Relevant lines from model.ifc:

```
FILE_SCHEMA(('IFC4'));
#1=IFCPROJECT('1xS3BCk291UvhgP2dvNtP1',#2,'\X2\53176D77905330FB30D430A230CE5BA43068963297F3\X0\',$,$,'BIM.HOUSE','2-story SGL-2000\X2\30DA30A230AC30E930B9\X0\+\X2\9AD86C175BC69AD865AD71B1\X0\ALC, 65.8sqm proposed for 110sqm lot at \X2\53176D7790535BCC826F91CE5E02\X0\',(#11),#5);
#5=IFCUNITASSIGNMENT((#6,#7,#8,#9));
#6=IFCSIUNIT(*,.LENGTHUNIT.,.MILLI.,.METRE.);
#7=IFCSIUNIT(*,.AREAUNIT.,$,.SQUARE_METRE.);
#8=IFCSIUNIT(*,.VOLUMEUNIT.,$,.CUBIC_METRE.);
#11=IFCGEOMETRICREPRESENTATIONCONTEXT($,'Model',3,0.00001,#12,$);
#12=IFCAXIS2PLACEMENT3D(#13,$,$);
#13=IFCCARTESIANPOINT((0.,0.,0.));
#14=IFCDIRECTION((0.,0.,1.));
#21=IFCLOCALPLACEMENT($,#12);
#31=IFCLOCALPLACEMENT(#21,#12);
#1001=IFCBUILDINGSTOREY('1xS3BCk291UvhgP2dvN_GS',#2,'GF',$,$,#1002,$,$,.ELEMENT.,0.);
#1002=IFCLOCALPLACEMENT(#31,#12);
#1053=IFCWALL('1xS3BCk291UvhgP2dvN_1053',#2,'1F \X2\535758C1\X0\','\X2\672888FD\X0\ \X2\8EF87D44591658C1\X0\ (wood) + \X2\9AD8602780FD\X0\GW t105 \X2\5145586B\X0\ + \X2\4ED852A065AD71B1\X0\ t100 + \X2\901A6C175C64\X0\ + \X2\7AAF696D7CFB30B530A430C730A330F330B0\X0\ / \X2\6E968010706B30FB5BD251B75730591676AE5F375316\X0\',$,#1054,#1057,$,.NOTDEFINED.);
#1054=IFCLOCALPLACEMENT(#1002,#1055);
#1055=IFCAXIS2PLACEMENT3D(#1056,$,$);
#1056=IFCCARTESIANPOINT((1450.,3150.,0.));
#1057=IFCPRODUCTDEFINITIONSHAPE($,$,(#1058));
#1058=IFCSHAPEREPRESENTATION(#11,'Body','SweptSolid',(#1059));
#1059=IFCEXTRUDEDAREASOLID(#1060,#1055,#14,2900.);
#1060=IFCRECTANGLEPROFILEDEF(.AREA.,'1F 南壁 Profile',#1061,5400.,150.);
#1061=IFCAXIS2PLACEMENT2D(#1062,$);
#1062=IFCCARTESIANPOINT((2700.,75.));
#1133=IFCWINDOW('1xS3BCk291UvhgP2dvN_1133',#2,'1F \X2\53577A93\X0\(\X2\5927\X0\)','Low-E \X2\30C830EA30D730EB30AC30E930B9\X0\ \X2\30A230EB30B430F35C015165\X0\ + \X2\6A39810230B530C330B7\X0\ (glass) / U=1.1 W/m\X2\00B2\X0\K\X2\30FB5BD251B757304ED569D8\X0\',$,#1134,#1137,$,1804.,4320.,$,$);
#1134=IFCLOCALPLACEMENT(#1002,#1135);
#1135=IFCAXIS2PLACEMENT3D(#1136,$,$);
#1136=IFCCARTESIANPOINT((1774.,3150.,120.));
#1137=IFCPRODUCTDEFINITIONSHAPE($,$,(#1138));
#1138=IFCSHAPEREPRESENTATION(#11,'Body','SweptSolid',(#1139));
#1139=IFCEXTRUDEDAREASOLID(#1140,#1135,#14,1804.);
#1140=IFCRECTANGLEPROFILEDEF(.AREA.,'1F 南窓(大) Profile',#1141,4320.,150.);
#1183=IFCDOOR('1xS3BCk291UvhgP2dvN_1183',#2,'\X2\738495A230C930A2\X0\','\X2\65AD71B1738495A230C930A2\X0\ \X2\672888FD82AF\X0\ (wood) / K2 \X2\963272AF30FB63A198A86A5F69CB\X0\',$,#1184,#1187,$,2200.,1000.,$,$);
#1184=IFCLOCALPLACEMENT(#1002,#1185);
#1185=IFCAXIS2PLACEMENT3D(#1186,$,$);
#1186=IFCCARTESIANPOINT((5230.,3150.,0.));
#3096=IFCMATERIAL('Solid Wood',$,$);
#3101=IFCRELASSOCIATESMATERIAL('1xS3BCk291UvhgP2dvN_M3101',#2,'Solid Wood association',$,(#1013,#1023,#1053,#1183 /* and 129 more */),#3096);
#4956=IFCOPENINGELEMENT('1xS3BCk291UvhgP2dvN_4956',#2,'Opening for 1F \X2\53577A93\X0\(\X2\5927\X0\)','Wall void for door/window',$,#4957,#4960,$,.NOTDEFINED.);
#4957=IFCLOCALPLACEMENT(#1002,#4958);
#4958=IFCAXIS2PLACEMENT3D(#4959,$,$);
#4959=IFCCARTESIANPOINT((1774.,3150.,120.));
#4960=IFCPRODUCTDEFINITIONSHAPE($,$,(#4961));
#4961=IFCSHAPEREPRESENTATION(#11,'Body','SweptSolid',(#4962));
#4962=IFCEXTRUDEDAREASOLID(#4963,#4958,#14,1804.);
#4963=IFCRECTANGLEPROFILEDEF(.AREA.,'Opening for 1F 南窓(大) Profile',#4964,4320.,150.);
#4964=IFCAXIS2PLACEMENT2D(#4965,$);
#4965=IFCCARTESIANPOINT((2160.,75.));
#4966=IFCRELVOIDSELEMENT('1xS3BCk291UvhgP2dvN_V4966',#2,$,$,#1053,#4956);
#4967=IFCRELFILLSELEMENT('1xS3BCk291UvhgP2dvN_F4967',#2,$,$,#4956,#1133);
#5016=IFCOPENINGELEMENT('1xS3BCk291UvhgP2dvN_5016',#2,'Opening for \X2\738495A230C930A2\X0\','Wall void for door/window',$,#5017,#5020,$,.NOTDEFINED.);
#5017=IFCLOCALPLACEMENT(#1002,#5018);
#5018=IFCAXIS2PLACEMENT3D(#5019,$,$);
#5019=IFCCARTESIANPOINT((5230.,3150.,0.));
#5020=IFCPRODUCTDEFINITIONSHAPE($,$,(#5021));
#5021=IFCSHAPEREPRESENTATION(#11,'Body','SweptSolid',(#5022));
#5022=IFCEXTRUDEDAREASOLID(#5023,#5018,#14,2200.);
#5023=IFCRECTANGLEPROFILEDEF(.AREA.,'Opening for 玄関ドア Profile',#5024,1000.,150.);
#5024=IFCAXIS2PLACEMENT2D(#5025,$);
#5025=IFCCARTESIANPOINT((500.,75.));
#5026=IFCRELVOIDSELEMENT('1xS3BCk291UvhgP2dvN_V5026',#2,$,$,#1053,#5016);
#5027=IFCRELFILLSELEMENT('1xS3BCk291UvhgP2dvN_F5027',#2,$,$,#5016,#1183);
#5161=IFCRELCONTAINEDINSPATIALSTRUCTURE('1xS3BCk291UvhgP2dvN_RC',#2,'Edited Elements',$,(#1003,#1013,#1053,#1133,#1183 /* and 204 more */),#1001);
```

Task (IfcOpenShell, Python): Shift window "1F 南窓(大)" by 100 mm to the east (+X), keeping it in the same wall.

```python
import ifcopenshell
import ifcopenshell.api.geometry
import ifcopenshell.util.placement

model = ifcopenshell.open("model.ifc")

window = model.by_guid("1xS3BCk291UvhgP2dvN_1133")
opening = window.FillsVoids[0].RelatingOpeningElement
wall = opening.VoidsElements[0].RelatingBuildingElement

wall_matrix = ifcopenshell.util.placement.get_local_placement(wall.ObjectPlacement)
shift = wall_matrix[:3, 0] * 100.0
before = ifcopenshell.util.placement.get_local_placement(window.ObjectPlacement)[:3, 3].copy()

# The window is not placed relative to its opening, so move both.
for product in (opening, window):
    matrix = ifcopenshell.util.placement.get_local_placement(product.ObjectPlacement)
    matrix[:3, 3] += shift
    ifcopenshell.api.geometry.edit_object_placement(model, product=product, matrix=matrix, is_si=False)

after = ifcopenshell.util.placement.get_local_placement(window.ObjectPlacement)[:3, 3]
print("window moved by", (after - before).round(3) + 0.0)

model.write("model_rev.ifc")
```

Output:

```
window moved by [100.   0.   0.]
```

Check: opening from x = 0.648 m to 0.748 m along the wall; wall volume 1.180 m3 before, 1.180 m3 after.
